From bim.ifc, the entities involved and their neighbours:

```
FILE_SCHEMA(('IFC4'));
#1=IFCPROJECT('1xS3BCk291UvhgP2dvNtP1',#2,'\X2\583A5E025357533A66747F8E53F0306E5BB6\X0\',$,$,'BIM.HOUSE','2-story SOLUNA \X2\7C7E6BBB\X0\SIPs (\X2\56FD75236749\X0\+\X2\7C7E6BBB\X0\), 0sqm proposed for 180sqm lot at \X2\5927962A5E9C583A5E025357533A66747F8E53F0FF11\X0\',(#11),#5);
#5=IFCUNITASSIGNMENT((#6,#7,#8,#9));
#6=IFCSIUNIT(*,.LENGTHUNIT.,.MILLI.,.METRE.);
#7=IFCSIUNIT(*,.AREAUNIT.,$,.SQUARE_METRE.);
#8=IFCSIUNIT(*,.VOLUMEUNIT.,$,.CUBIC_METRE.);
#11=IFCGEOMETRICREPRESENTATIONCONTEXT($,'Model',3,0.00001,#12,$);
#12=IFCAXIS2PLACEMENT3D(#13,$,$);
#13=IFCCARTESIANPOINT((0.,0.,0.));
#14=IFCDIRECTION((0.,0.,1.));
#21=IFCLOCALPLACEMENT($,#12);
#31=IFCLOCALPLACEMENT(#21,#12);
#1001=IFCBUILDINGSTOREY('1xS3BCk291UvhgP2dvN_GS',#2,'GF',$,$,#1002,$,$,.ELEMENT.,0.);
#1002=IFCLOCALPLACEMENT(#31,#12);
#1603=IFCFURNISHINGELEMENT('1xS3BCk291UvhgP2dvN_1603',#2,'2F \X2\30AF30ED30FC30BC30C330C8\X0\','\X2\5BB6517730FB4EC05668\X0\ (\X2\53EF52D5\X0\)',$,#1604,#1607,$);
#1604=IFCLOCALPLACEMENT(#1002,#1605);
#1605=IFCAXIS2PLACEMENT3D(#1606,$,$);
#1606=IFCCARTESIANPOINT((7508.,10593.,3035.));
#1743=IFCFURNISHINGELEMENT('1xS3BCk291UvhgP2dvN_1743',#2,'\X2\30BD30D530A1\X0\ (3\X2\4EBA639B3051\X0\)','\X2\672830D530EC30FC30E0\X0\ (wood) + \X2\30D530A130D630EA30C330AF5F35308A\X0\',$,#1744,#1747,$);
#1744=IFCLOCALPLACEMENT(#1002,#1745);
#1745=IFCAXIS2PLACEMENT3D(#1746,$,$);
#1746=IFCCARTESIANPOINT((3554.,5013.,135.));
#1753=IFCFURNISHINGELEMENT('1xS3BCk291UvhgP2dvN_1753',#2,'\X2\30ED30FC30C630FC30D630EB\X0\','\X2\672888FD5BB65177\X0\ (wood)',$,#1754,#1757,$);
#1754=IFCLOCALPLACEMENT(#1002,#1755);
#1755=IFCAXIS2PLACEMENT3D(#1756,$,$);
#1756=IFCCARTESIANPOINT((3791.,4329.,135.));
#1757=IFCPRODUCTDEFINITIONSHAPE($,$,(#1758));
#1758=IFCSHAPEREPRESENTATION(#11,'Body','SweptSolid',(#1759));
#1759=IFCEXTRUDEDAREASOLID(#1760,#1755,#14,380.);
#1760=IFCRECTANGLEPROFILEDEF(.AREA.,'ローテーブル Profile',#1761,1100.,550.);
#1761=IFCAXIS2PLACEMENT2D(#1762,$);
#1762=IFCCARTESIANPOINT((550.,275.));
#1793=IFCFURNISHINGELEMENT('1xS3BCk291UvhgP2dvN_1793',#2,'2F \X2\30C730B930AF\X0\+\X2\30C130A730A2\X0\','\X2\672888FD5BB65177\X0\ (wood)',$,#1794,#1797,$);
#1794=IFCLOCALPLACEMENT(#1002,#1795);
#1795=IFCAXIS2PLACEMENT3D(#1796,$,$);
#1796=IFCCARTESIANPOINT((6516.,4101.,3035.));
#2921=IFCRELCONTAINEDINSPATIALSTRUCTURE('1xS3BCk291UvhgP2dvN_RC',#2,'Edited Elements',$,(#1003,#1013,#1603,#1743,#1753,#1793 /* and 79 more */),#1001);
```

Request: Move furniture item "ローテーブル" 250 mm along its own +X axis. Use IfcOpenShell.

```python
import ifcopenshell
import ifcopenshell.api.geometry
import ifcopenshell.util.placement
import ifcopenshell.util.unit

model = ifcopenshell.open("bim.ifc")
unit_scale = ifcopenshell.util.unit.calculate_unit_scale(model)

item = model.by_id(1753)
matrix = ifcopenshell.util.placement.get_local_placement(item.ObjectPlacement)
matrix[:3, 3] += matrix[:3, 0] * 0.25 / unit_scale
ifcopenshell.api.geometry.edit_object_placement(model, product=item, matrix=matrix, is_si=False)

print(ifcopenshell.util.placement.get_local_placement(item.ObjectPlacement).round(3) + 0.0)

model.write("bim_updated.ifc")
```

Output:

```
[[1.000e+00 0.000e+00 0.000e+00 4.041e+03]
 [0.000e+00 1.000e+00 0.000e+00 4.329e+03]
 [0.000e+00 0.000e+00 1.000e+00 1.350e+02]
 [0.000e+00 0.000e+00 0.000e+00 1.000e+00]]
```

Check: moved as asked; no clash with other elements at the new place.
